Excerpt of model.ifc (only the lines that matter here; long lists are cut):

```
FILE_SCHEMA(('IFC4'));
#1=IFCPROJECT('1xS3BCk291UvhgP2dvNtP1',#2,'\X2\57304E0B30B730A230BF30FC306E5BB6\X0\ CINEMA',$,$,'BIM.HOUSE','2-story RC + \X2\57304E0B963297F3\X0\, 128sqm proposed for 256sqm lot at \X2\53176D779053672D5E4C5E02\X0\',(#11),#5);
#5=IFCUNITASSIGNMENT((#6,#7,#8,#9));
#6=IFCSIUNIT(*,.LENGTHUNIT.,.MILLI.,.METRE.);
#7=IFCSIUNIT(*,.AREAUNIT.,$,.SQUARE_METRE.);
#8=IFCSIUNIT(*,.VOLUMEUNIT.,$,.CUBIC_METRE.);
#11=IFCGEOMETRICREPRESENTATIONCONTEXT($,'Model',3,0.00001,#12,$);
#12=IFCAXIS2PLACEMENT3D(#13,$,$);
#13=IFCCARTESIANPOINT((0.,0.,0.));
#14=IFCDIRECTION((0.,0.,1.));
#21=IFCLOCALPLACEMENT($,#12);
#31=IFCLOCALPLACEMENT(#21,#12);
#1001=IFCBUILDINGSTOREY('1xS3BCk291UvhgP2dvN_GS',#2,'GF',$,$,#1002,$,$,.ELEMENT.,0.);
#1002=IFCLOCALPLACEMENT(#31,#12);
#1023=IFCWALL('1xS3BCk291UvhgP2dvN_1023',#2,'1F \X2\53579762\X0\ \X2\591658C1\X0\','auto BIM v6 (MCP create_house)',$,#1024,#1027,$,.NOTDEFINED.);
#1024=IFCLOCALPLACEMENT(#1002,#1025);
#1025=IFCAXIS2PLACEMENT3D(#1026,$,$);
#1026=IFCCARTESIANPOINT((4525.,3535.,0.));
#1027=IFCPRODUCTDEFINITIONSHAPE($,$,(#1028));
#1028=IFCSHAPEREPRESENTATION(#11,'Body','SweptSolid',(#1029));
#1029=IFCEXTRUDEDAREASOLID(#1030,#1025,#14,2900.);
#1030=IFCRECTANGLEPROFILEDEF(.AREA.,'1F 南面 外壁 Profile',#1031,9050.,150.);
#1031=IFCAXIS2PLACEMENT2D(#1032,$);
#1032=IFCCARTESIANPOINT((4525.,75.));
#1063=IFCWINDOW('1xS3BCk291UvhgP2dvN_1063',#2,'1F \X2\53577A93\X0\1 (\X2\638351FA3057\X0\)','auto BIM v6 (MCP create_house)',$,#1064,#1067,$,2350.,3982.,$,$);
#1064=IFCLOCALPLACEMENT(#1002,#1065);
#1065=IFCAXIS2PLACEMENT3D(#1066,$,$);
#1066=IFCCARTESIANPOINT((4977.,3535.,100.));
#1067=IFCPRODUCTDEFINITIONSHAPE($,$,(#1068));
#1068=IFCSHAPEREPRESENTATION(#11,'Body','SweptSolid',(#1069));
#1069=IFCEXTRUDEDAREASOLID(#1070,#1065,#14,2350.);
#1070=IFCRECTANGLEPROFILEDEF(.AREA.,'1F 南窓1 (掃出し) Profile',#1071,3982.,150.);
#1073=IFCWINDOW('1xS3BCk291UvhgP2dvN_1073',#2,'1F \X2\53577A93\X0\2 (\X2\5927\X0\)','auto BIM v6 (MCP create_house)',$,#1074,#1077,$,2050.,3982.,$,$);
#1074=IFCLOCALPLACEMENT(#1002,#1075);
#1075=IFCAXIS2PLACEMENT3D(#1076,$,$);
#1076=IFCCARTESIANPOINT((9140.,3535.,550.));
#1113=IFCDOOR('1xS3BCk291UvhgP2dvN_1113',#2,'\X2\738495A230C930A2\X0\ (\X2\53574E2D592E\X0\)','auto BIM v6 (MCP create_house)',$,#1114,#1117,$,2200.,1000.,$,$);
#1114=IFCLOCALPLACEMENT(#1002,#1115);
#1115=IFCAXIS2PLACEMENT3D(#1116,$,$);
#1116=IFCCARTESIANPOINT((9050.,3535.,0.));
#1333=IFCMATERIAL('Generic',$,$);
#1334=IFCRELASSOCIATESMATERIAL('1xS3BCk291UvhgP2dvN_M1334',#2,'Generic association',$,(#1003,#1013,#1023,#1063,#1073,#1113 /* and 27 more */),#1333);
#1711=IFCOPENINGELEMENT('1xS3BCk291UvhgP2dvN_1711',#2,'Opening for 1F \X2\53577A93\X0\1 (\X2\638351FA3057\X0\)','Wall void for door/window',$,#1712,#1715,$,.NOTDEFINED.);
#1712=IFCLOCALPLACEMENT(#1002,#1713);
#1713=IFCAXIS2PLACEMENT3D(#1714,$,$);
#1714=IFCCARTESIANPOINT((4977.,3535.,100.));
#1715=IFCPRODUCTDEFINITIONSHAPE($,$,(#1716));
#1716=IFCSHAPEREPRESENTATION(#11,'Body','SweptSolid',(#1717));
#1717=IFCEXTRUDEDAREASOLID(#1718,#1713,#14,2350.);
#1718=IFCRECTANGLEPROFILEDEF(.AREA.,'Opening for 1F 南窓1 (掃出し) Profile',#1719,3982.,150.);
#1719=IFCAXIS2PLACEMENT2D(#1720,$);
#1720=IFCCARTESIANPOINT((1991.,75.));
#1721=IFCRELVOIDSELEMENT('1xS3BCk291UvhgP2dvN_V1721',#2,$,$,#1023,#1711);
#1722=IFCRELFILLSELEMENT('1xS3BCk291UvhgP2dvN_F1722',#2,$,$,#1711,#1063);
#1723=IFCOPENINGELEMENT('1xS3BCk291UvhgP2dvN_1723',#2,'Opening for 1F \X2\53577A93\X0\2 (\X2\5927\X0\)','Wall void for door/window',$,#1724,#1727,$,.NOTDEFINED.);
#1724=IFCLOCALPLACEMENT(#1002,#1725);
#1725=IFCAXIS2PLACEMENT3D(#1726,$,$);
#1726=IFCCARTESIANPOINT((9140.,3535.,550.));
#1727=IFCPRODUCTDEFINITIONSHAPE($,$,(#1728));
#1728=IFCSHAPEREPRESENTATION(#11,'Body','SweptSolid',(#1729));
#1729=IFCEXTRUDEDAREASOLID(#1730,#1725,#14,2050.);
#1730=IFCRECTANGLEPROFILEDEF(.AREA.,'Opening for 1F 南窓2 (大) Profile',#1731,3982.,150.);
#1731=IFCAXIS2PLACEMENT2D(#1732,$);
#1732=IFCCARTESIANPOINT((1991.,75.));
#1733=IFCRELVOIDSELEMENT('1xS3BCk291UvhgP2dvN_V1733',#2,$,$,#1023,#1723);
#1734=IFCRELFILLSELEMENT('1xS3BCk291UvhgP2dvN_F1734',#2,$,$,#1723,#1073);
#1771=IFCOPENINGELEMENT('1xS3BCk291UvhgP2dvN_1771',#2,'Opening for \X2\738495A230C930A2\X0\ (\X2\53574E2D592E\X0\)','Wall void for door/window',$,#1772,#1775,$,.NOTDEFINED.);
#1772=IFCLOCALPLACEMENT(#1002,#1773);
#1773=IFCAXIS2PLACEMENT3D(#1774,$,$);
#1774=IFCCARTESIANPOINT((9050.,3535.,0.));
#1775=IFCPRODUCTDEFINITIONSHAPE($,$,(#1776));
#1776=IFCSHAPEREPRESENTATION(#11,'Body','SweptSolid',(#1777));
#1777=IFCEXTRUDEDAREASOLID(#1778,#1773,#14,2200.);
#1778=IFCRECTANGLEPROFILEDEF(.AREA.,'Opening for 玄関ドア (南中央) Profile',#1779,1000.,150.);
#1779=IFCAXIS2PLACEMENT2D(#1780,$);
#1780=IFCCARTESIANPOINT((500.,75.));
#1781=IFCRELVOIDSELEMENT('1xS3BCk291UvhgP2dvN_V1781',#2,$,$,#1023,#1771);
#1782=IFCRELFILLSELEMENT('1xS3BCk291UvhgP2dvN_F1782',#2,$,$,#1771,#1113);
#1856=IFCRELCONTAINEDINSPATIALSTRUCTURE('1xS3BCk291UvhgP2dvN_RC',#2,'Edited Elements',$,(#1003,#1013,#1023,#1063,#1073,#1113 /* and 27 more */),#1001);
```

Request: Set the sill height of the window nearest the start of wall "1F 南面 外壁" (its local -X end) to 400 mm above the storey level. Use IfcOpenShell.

```python
import numpy as np
import ifcopenshell
import ifcopenshell.api.geometry
import ifcopenshell.geom
import ifcopenshell.util.element
import ifcopenshell.util.placement
import ifcopenshell.util.shape
import ifcopenshell.util.unit

model = ifcopenshell.open("model.ifc")
unit_scale = ifcopenshell.util.unit.calculate_unit_scale(model)

window = model.by_guid("1xS3BCk291UvhgP2dvN_1063")
opening = window.FillsVoids[0].RelatingOpeningElement
storey = ifcopenshell.util.element.get_container(window, ifc_class="IfcBuildingStorey")
level = ifcopenshell.util.placement.get_local_placement(storey.ObjectPlacement)[2, 3]

# The opening's origin need not be at the sill, so measure its lowest point.
shape = ifcopenshell.geom.create_shape(ifcopenshell.geom.settings(), opening)
bottom = ifcopenshell.util.shape.get_shape_bottom_elevation(shape, shape.geometry) / unit_scale
dz = level + 400.0 - bottom

shift = np.array([0.0, 0.0, dz])
# The window is not placed relative to its opening, so move both.
for product in (opening, window):
    matrix = ifcopenshell.util.placement.get_local_placement(product.ObjectPlacement)
    matrix[:3, 3] += shift
    ifcopenshell.api.geometry.edit_object_placement(model, product=product, matrix=matrix, is_si=False)

print(f"moved by {dz * unit_scale:+.3f} m")

model.write("model_v2.ifc")
```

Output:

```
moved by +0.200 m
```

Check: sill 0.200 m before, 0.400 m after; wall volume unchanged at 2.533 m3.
